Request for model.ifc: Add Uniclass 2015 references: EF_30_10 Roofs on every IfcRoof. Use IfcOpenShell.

First a look at what the model holds.

```python
import ifcopenshell

model = ifcopenshell.open("model.ifc")
print(model.schema)
print("classifications:", [c.Name for c in model.by_type("IfcClassification")])
for ifc_class in ("IfcDoor", "IfcRoof", "IfcStair", "IfcWall", "IfcWindow"):
    print(ifc_class, len(model.by_type(ifc_class)))
```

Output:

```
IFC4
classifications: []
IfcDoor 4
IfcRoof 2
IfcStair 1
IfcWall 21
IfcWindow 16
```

```python
import ifcopenshell
import ifcopenshell.api.classification

model = ifcopenshell.open("model.ifc")

system = ifcopenshell.api.classification.add_classification(model, classification="Uniclass 2015")

codes = {
    "IfcRoof": ("EF_30_10", "Roofs"),
}
for ifc_class, (code, name) in codes.items():
    products = model.by_type(ifc_class)
    ifcopenshell.api.classification.add_reference(
        model, products=products, classification=system, identification=code, name=name
    )
    print(code, len(products))

model.write("model_v2.ifc")
```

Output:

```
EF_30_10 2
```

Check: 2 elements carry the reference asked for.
